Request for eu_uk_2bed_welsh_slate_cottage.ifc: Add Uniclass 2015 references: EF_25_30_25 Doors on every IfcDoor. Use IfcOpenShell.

First a look at what the model holds.

```python
import ifcopenshell

model = ifcopenshell.open("eu_uk_2bed_welsh_slate_cottage.ifc")
print(model.schema)
print("classifications:", [c.Name for c in model.by_type("IfcClassification")])
for ifc_class in ("IfcDoor", "IfcRoof", "IfcStair", "IfcWall", "IfcWindow"):
    print(ifc_class, len(model.by_type(ifc_class)))
```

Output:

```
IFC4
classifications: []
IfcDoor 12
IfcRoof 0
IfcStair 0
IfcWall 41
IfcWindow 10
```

```python
import ifcopenshell
import ifcopenshell.api.classification

model = ifcopenshell.open("eu_uk_2bed_welsh_slate_cottage.ifc")

system = ifcopenshell.api.classification.add_classification(model, classification="Uniclass 2015")

codes = {
    "IfcDoor": ("EF_25_30_25", "Doors"),
}
for ifc_class, (code, name) in codes.items():
    products = model.by_type(ifc_class)
    ifcopenshell.api.classification.add_reference(
        model, products=products, classification=system, identification=code, name=name
    )
    print(code, len(products))

model.write("eu_uk_2bed_welsh_slate_cottage_updated.ifc")
```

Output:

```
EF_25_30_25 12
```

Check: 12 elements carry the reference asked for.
